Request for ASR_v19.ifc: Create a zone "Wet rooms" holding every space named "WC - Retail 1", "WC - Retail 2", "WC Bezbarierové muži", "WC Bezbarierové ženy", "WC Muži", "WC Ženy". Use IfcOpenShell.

First a look at what the model holds.

```python
import ifcopenshell

model = ifcopenshell.open("ASR_v19.ifc")
print(model.schema)
seen = {}
for space in model.by_type("IfcSpace"):
    seen[space.LongName] = seen.get(space.LongName, 0) + 1
for name, count in sorted(seen.items(), key=str):
    print(count, "x", name)
print("zones:", [z.Name for z in model.by_type("IfcZone")][:20])
```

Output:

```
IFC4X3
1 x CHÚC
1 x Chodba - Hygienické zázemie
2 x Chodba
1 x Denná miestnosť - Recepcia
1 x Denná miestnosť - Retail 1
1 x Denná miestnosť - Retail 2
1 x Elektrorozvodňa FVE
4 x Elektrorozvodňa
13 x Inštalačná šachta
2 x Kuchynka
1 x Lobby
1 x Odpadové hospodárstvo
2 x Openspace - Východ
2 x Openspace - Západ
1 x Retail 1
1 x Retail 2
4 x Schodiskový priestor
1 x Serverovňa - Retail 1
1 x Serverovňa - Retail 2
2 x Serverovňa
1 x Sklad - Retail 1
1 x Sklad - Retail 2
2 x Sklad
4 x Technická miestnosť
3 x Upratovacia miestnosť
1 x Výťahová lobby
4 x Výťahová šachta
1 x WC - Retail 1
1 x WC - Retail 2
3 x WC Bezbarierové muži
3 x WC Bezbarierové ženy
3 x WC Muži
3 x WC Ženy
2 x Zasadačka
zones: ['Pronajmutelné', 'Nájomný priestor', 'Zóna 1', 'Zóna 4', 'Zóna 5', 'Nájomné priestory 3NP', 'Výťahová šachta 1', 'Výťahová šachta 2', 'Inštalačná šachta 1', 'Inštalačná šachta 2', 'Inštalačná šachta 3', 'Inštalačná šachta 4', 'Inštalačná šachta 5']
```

```python
import ifcopenshell
import ifcopenshell.api.group
import ifcopenshell.api.root

model = ifcopenshell.open("ASR_v19.ifc")

names = {"WC - Retail 1", "WC - Retail 2", "WC Bezbarierové muži", "WC Bezbarierové ženy", "WC Muži", "WC Ženy"}
spaces = [s for s in model.by_type("IfcSpace") if s.LongName in names]

zone = ifcopenshell.api.root.create_entity(model, ifc_class="IfcZone", name="Wet rooms")
ifcopenshell.api.group.assign_group(model, products=spaces, group=zone)
print(len(spaces), "spaces in", zone.Name)

model.write("ASR_v19_v2.ifc")
```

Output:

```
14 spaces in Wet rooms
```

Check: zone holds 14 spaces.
